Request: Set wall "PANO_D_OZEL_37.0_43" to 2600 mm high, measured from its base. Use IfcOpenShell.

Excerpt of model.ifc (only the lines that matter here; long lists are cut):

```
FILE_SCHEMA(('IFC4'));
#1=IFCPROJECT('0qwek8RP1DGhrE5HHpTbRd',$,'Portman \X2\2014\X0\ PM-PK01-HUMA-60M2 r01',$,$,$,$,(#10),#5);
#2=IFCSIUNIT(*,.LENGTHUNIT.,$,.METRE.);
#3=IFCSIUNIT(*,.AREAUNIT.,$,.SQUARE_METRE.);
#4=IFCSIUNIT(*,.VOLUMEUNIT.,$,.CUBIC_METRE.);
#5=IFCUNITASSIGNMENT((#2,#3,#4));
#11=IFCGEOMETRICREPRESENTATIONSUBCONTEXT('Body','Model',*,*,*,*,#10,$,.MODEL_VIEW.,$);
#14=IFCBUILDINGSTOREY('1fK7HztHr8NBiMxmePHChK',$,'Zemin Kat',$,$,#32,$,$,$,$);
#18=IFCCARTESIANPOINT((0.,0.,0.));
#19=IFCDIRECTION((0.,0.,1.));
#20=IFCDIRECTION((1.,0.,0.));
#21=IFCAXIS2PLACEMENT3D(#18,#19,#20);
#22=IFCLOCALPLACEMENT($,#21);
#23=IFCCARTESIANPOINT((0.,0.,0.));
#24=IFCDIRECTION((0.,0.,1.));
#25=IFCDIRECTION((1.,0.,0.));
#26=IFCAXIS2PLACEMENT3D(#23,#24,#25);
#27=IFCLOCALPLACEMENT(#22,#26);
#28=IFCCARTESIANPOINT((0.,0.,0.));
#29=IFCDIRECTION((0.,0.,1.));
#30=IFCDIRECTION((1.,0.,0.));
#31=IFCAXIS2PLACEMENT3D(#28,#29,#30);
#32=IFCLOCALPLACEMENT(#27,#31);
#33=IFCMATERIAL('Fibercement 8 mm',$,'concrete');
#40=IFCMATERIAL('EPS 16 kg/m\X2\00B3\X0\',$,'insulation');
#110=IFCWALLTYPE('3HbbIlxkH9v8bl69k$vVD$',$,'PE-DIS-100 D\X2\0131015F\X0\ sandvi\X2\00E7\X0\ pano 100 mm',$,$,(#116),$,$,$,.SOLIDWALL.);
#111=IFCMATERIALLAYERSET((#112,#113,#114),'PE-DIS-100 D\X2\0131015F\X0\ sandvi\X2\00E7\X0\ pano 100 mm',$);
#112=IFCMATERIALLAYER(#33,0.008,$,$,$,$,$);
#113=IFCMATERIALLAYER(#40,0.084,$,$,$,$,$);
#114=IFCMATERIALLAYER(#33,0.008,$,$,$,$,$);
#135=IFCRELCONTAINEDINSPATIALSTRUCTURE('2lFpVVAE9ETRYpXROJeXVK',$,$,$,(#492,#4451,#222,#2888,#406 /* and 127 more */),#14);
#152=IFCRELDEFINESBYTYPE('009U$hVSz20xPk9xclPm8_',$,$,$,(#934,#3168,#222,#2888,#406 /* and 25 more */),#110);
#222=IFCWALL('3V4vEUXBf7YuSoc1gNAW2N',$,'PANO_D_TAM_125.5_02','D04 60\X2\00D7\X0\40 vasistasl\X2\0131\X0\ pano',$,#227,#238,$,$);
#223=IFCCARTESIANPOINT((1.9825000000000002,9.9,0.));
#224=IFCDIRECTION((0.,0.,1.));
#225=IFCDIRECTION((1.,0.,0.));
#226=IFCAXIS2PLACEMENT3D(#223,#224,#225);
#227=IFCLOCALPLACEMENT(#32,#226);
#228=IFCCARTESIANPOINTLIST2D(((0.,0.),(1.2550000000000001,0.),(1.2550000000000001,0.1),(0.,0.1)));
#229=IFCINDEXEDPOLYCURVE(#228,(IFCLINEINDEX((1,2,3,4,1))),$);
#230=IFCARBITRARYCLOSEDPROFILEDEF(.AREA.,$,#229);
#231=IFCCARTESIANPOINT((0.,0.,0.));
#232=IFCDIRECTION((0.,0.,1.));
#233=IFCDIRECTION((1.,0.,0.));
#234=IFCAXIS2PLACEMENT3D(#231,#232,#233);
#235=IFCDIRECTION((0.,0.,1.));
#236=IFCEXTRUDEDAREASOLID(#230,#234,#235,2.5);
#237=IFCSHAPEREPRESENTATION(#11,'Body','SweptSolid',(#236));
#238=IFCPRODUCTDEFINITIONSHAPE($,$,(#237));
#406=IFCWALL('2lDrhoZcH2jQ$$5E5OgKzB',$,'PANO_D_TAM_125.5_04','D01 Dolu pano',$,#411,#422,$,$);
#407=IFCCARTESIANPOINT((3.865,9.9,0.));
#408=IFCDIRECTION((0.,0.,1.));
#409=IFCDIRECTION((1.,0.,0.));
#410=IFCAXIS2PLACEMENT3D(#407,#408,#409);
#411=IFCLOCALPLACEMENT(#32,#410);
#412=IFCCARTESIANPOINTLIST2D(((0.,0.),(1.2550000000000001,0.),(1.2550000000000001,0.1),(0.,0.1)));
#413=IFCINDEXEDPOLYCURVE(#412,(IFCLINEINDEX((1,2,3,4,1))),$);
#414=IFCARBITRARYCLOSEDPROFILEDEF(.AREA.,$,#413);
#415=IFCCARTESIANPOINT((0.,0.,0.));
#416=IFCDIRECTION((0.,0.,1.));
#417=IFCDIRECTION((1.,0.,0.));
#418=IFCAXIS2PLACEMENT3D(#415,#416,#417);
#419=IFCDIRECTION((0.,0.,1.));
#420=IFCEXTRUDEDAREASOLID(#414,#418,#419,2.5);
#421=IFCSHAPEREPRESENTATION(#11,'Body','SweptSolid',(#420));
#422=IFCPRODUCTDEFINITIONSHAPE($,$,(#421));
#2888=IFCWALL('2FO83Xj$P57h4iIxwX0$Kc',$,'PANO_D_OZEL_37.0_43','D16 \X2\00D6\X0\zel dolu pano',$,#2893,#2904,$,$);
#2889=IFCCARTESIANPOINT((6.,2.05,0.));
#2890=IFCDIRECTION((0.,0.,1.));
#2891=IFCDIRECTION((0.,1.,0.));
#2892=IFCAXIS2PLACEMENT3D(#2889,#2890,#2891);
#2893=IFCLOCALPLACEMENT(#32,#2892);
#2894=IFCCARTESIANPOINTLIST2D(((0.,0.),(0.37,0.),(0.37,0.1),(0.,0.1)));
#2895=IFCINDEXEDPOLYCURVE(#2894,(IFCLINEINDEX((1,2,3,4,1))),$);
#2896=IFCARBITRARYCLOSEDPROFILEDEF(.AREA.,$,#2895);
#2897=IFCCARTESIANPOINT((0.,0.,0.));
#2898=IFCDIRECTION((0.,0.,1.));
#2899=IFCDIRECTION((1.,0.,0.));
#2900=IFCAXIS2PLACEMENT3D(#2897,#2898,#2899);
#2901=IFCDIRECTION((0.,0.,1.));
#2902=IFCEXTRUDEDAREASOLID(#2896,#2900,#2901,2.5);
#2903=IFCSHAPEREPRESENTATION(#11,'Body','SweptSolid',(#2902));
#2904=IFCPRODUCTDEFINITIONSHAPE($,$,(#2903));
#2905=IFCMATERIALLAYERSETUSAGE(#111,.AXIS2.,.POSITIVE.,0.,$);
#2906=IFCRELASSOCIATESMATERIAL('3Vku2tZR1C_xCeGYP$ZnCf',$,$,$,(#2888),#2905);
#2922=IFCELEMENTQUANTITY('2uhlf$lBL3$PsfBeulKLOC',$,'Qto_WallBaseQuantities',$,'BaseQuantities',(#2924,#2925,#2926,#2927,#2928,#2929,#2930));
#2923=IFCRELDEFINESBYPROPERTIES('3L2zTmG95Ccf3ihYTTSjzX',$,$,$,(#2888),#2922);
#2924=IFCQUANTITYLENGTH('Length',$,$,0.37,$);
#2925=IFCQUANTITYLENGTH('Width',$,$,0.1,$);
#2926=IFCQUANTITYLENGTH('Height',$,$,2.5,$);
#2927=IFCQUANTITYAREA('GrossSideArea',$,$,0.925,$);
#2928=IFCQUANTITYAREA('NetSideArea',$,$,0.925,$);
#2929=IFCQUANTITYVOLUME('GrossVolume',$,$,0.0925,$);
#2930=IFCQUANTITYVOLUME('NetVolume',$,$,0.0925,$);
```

```python
import ifcopenshell
import ifcopenshell.api.pset
import ifcopenshell.geom
import ifcopenshell.util.element
import ifcopenshell.util.representation
import ifcopenshell.util.shape
import ifcopenshell.util.unit

model = ifcopenshell.open("model.ifc")
unit_scale = ifcopenshell.util.unit.calculate_unit_scale(model)
area_scale = ifcopenshell.util.unit.calculate_unit_scale(model, "AREAUNIT")
volume_scale = ifcopenshell.util.unit.calculate_unit_scale(model, "VOLUMEUNIT")
settings = ifcopenshell.geom.settings()


def volume(element):
    """Net volume in cubic metres, openings subtracted."""
    shape = ifcopenshell.geom.create_shape(settings, element)
    return ifcopenshell.util.shape.get_volume(shape.geometry)


wall = model.by_guid("2FO83Xj$P57h4iIxwX0$Kc")
before = volume(wall)

body = ifcopenshell.util.representation.get_representation(wall, "Model", "Body")
solid = body.Items[0]
old_height = solid.Depth
solid.Depth = 2.6 / unit_scale
after = volume(wall)
thickness = 0.1  # wall thickness in metres

# Update the stored height, areas and volumes.
qto = model.by_id(ifcopenshell.util.element.get_pset(wall, "Qto_WallBaseQuantities", should_inherit=False)["id"])
ifcopenshell.api.pset.edit_qto(model, qto=qto, properties={
    "Height": solid.Depth,
    "GrossSideArea": ifcopenshell.util.element.get_pset(wall, "Qto_WallBaseQuantities", "GrossSideArea") * solid.Depth / old_height,
    "NetSideArea": after / thickness / area_scale,
    "GrossVolume": ifcopenshell.util.element.get_pset(wall, "Qto_WallBaseQuantities", "GrossVolume") * solid.Depth / old_height,
    "NetVolume": after / volume_scale,
})

print(f"height {old_height:g} -> {solid.Depth:g}, volume {before:.3f} -> {after:.3f} m3")

model.write("model_edited.ifc")
```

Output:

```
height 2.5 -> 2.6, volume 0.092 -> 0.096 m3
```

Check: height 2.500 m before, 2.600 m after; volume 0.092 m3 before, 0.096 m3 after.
